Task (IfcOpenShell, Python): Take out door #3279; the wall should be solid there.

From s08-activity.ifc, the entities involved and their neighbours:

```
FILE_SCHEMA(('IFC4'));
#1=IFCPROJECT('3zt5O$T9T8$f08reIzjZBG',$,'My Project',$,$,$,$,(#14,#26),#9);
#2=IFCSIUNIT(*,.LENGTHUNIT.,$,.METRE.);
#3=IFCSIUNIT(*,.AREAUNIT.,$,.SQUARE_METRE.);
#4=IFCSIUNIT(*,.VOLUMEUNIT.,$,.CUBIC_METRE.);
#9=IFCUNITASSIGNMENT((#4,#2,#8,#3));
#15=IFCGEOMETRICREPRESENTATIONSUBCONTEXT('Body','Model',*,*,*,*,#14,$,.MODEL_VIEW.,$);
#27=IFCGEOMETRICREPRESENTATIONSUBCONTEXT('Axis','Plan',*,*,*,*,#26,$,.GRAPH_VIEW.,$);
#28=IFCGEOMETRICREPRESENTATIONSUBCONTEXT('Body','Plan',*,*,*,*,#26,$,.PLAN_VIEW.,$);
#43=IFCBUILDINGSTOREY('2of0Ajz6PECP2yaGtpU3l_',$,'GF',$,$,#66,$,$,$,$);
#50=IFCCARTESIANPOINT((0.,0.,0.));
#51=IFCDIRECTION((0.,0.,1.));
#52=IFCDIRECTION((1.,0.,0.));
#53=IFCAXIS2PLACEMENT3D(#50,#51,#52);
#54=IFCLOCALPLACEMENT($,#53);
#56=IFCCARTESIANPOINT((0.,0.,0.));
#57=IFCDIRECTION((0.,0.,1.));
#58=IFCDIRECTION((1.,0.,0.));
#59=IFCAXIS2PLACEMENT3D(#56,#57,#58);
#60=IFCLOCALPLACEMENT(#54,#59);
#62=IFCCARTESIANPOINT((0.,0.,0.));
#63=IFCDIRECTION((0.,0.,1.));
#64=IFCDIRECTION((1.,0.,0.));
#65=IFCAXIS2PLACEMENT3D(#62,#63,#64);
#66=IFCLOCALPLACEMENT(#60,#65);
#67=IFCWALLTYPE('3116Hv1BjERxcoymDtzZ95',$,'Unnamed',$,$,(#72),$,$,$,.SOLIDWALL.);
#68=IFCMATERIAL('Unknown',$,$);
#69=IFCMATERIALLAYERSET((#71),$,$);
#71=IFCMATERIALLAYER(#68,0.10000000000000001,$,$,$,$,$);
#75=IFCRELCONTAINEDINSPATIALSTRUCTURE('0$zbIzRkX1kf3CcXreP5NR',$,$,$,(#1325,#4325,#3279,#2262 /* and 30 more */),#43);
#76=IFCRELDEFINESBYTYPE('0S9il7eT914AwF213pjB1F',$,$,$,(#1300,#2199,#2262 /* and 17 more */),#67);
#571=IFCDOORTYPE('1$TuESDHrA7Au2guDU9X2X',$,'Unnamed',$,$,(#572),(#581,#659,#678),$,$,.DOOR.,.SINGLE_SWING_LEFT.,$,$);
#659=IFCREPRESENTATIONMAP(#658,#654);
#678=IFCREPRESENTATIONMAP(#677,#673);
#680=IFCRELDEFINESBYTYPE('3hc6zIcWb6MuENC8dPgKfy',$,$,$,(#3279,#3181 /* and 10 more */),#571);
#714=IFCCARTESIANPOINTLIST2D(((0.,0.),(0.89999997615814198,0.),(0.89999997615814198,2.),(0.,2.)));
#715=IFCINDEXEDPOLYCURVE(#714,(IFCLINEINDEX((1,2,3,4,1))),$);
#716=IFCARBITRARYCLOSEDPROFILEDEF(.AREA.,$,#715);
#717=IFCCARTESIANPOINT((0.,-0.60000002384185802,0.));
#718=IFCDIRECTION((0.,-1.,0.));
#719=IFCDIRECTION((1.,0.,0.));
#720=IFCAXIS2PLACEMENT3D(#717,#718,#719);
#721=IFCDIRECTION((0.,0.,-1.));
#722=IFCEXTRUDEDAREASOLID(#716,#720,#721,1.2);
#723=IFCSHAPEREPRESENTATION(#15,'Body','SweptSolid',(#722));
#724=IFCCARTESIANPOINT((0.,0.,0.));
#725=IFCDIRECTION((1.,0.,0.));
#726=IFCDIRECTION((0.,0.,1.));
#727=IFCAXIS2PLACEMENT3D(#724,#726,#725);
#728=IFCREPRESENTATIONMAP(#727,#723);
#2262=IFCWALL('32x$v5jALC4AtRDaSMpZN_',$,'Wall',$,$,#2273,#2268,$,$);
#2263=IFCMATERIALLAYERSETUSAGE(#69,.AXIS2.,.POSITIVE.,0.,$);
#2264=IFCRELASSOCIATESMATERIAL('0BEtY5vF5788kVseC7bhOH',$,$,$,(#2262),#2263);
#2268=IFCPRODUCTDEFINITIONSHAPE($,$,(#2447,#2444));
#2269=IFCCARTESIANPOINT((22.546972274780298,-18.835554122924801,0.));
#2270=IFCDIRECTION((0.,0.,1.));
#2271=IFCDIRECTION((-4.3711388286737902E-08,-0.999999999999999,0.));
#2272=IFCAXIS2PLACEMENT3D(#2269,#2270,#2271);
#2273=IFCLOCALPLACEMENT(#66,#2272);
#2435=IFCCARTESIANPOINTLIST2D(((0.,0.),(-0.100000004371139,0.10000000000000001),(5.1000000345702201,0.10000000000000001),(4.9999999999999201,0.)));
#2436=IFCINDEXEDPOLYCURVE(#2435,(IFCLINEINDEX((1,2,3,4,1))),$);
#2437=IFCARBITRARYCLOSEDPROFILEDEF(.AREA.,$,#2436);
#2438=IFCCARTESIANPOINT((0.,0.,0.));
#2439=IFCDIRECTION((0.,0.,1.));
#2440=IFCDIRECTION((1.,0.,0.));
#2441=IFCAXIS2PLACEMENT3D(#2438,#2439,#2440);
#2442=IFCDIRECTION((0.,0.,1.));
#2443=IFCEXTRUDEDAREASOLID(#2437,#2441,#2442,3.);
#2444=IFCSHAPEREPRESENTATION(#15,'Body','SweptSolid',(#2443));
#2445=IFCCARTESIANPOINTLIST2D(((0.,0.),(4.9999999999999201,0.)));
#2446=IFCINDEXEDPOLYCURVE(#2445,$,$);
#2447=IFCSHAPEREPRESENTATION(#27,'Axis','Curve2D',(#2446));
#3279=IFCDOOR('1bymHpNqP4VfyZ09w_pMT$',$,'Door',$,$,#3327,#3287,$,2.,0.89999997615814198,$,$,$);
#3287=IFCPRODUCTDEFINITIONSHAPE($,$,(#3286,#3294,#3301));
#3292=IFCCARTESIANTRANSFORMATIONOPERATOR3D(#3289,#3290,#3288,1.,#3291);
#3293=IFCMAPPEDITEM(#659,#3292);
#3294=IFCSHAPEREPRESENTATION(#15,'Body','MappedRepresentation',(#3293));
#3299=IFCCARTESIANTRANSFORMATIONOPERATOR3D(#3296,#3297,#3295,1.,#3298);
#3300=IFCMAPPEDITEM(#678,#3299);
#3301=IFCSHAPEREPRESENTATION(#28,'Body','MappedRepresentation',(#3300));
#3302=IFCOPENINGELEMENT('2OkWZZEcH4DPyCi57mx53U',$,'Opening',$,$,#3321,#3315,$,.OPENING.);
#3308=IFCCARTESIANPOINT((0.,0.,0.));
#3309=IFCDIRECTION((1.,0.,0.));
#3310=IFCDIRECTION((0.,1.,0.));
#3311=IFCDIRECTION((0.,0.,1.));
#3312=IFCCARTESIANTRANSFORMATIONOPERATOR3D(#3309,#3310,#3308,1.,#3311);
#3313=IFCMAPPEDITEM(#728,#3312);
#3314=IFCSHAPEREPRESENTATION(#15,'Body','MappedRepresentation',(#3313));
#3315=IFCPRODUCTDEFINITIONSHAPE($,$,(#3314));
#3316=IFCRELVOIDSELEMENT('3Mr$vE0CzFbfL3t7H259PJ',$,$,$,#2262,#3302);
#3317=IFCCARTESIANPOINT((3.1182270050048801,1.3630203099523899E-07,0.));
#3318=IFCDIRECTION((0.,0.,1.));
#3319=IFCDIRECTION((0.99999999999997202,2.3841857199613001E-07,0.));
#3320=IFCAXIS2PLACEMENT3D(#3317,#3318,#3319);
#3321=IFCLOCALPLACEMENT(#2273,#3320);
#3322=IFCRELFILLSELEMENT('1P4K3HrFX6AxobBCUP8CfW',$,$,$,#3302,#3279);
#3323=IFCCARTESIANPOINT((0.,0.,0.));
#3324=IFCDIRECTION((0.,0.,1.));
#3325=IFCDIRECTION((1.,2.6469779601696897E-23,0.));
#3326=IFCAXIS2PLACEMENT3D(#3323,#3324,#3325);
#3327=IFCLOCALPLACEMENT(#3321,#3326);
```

```python
import ifcopenshell
import ifcopenshell.api.feature
import ifcopenshell.api.root
import ifcopenshell.geom
import ifcopenshell.util.shape

model = ifcopenshell.open("s08-activity.ifc")
settings = ifcopenshell.geom.settings()


def volume(element):
    """Net volume in cubic metres, openings subtracted."""
    shape = ifcopenshell.geom.create_shape(settings, element)
    return ifcopenshell.util.shape.get_volume(shape.geometry)


door = model.by_guid("1bymHpNqP4VfyZ09w_pMT$")
opening = door.FillsVoids[0].RelatingOpeningElement
wall = opening.VoidsElements[0].RelatingBuildingElement
before = volume(wall)

ifcopenshell.api.root.remove_product(model, product=door)
ifcopenshell.api.feature.remove_feature(model, feature=opening)

after = volume(wall)

print(f"wall volume {before:.3f} -> {after:.3f} m3")

model.write("s08-activity_edited.ifc")
```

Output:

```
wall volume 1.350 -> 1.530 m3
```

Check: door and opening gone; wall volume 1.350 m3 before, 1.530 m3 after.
